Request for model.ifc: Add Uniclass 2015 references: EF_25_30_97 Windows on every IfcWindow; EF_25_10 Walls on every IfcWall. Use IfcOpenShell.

First a look at what the model holds.

```python
import ifcopenshell

model = ifcopenshell.open("model.ifc")
print(model.schema)
print("classifications:", [c.Name for c in model.by_type("IfcClassification")])
for ifc_class in ("IfcDoor", "IfcRoof", "IfcStair", "IfcWall", "IfcWindow"):
    print(ifc_class, len(model.by_type(ifc_class)))
```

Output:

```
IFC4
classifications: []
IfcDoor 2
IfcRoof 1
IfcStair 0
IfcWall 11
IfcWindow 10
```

```python
import ifcopenshell
import ifcopenshell.api.classification

model = ifcopenshell.open("model.ifc")

system = ifcopenshell.api.classification.add_classification(model, classification="Uniclass 2015")

codes = {
    "IfcWindow": ("EF_25_30_97", "Windows"),
    "IfcWall": ("EF_25_10", "Walls"),
}
for ifc_class, (code, name) in codes.items():
    products = model.by_type(ifc_class)
    ifcopenshell.api.classification.add_reference(
        model, products=products, classification=system, identification=code, name=name
    )
    print(code, len(products))

model.write("model_updated.ifc")
```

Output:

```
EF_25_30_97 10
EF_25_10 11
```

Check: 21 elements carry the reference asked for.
